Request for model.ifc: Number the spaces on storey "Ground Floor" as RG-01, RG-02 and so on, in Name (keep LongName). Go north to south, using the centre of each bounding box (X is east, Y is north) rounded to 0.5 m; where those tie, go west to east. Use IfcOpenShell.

First a look at what the model holds.

```python
import ifcopenshell
import ifcopenshell.util.element
import ifcopenshell.util.placement

model = ifcopenshell.open("model.ifc")
print(model.schema)
storey = next(s for s in model.by_type("IfcBuildingStorey") if s.Name == "Ground Floor")
spaces = [e for e in ifcopenshell.util.element.get_decomposition(storey) if e.is_a("IfcSpace")]
for e in sorted(spaces, key=lambda e: e.id()):
    origin = ifcopenshell.util.placement.get_local_placement(e.ObjectPlacement)[:3, 3]
    print(e.id(), e.Name, e.LongName, origin.round(2) + 0.0, sep=" | ")
```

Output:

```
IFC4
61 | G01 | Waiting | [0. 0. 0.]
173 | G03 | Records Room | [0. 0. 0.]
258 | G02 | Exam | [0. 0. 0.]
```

```python
import ifcopenshell
import ifcopenshell.geom
import ifcopenshell.util.element
import ifcopenshell.util.shape

model = ifcopenshell.open("model.ifc")
settings = ifcopenshell.geom.settings()
settings.set("use-world-coords", True)


def centre(element):
    shape = ifcopenshell.geom.create_shape(settings, element)
    return ifcopenshell.util.shape.get_bbox_centroid(shape.geometry)


storey = next(s for s in model.by_type("IfcBuildingStorey") if s.Name == "Ground Floor")
spaces = [e for e in ifcopenshell.util.element.get_decomposition(storey) if e.is_a("IfcSpace")]

# Insertion points can sit at a corner or the storey origin, so sort by the geometry (in metres).
centres = {e: centre(e) for e in spaces}
spaces.sort(key=lambda e: (-round(centres[e][1] / 0.5), centres[e][0]))

for i, e in enumerate(spaces, start=1):
    number = f"RG-{i:02d}"
    e.Name = number
    print(e.id(), number)

model.write("model_rev.ifc")
```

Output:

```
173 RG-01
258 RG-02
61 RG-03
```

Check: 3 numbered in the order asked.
